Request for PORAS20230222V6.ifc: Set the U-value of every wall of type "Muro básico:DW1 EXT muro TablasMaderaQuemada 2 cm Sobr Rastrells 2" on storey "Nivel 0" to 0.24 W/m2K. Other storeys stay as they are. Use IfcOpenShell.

First a look at what the model holds.

```python
import ifcopenshell
import ifcopenshell.util.element

model = ifcopenshell.open("PORAS20230222V6.ifc")
print(model.schema)
storey = next(s for s in model.by_type("IfcBuildingStorey") if s.Name == "Nivel 0")
walls = [e for e in ifcopenshell.util.element.get_decomposition(storey) if e.is_a("IfcWall")]
seen = {}
for e in walls:
    element_type = ifcopenshell.util.element.get_type(e)
    key = (element_type.Name if element_type != e and element_type else None, ifcopenshell.util.element.get_pset(e, "Pset_WallCommon", "ThermalTransmittance"))
    seen[key] = seen.get(key, 0) + 1
for (name, value), count in sorted(seen.items(), key=str):
    print(count, "x", name, "|", value)
```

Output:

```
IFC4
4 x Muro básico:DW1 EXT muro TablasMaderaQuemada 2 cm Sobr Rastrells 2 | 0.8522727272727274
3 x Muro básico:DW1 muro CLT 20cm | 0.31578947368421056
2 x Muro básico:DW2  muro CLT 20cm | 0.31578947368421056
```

```python
import ifcopenshell
import ifcopenshell.api.pset
import ifcopenshell.util.element

model = ifcopenshell.open("PORAS20230222V6.ifc")

storey = next(s for s in model.by_type("IfcBuildingStorey") if s.Name == "Nivel 0")
walls = [e for e in ifcopenshell.util.element.get_decomposition(storey) if e.is_a("IfcWall")]

count = 0
for e in walls:
    element_type = ifcopenshell.util.element.get_type(e)
    if element_type in (None, e) or element_type.Name != "Muro básico:DW1 EXT muro TablasMaderaQuemada 2 cm Sobr Rastrells 2":
        continue
    # add_pset returns the element's existing set when there is one.
    pset = ifcopenshell.api.pset.add_pset(model, product=e, name="Pset_WallCommon")
    ifcopenshell.api.pset.edit_pset(model, pset=pset, properties={"ThermalTransmittance": 0.24})
    count += 1

print(count, "walls updated")

model.write("PORAS20230222V6-out.ifc")
```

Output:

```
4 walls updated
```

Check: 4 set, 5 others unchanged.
